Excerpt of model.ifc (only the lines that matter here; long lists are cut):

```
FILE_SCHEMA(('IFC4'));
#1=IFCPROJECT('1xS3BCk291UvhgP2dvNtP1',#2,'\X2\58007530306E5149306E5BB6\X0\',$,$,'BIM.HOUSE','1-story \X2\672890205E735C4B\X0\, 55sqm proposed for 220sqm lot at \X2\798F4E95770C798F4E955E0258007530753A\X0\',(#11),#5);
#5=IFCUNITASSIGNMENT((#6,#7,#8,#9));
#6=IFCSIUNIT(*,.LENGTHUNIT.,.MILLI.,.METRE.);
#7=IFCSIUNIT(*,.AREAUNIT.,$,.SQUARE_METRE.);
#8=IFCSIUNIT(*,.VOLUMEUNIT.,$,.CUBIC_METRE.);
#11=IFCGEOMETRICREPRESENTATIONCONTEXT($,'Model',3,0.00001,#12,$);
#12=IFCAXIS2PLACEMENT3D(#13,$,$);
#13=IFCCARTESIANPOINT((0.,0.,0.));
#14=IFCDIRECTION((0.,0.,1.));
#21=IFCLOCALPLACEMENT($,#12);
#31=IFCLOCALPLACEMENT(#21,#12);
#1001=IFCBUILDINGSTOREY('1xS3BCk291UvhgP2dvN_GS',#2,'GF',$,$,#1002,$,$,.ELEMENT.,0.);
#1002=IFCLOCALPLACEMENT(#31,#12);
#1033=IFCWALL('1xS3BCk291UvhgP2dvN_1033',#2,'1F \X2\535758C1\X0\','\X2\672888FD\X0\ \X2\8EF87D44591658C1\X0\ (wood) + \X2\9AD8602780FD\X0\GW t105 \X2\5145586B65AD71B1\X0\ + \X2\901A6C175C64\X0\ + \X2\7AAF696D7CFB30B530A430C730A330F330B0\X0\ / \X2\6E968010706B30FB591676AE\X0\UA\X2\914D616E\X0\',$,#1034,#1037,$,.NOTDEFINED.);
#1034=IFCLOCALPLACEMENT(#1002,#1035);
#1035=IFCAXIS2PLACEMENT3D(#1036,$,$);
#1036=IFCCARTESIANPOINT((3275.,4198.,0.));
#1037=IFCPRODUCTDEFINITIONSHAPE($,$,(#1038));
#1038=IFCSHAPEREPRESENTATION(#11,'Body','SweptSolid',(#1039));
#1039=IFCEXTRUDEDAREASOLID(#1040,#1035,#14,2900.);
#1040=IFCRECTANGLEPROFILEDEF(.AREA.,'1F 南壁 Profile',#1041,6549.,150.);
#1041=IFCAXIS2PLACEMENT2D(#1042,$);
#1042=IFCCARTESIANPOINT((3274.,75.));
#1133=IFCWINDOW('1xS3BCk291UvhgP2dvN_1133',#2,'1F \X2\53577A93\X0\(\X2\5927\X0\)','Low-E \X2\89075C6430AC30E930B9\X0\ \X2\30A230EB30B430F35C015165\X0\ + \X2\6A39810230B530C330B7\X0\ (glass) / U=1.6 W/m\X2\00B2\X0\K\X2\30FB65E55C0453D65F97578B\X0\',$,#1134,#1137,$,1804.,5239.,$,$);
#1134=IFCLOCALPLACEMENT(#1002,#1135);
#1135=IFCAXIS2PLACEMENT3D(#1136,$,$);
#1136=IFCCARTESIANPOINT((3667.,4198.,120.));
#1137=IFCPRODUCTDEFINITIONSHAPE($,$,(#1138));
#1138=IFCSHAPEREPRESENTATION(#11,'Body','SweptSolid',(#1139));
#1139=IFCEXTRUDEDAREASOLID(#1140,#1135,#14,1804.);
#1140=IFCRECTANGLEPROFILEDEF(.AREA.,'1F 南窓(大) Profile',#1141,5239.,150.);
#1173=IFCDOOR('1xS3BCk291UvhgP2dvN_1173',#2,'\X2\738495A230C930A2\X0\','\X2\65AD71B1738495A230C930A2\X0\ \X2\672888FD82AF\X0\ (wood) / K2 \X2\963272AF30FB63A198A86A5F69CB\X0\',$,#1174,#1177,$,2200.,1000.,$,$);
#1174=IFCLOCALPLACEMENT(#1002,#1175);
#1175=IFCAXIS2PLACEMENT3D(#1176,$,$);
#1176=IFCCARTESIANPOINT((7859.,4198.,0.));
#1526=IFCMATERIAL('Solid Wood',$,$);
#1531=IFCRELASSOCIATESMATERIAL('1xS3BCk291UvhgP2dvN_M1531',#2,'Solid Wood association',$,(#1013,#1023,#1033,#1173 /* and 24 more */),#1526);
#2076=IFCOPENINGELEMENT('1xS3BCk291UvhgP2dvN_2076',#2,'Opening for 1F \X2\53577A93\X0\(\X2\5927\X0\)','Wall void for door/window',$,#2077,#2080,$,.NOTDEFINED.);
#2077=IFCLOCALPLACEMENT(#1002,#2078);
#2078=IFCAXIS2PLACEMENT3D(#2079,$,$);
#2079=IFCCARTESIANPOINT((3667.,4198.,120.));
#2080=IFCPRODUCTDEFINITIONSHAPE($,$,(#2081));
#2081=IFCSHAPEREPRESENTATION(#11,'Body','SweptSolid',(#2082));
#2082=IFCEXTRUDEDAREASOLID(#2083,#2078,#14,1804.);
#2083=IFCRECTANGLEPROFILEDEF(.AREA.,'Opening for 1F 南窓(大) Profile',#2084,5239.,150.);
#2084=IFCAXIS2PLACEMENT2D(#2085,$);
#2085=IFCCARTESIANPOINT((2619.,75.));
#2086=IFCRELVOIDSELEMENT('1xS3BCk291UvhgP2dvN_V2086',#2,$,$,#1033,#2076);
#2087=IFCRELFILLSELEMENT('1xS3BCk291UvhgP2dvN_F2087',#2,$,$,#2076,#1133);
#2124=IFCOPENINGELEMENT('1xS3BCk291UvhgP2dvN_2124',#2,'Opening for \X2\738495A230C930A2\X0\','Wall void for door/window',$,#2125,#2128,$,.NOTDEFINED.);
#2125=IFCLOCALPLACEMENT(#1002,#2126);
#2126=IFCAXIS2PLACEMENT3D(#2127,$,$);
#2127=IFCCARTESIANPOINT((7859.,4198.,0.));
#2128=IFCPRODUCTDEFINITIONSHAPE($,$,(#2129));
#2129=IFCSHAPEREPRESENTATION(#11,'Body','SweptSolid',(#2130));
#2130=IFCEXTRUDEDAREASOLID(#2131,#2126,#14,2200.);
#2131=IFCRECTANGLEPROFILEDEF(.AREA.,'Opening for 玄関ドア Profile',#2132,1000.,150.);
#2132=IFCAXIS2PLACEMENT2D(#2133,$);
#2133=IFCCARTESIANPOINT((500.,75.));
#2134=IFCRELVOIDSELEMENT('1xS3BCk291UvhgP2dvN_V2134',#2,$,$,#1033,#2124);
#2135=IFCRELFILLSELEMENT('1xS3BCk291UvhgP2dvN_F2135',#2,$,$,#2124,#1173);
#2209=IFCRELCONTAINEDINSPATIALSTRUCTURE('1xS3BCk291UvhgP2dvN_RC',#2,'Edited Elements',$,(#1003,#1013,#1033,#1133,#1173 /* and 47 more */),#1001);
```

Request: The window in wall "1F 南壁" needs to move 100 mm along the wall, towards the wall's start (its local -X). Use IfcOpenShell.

```python
import ifcopenshell
import ifcopenshell.api.geometry
import ifcopenshell.util.placement
import ifcopenshell.util.unit

model = ifcopenshell.open("model.ifc")
unit_scale = ifcopenshell.util.unit.calculate_unit_scale(model)

window = model.by_guid("1xS3BCk291UvhgP2dvN_1133")
opening = window.FillsVoids[0].RelatingOpeningElement
wall = opening.VoidsElements[0].RelatingBuildingElement

wall_matrix = ifcopenshell.util.placement.get_local_placement(wall.ObjectPlacement)
shift = wall_matrix[:3, 0] * -0.1 / unit_scale
before = ifcopenshell.util.placement.get_local_placement(window.ObjectPlacement)[:3, 3].copy()

# The window is not placed relative to its opening, so move both.
for product in (opening, window):
    matrix = ifcopenshell.util.placement.get_local_placement(product.ObjectPlacement)
    matrix[:3, 3] += shift
    ifcopenshell.api.geometry.edit_object_placement(model, product=product, matrix=matrix, is_si=False)

after = ifcopenshell.util.placement.get_local_placement(window.ObjectPlacement)[:3, 3]
print("window moved by", (after - before).round(3) + 0.0)

model.write("model_edited.ifc")
```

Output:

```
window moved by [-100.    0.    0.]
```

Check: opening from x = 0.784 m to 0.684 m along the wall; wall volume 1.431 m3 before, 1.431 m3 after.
